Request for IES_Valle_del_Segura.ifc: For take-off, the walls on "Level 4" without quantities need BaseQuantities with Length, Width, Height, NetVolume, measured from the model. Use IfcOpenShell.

First a look at what the model holds.

```python
import ifcopenshell
import ifcopenshell.util.element
import ifcopenshell.util.unit

model = ifcopenshell.open("IES_Valle_del_Segura.ifc")
print(model.schema)
for unit_type in ("LENGTHUNIT", "AREAUNIT", "VOLUMEUNIT"):
    print(unit_type, ifcopenshell.util.unit.calculate_unit_scale(model, unit_type))
storey = next(s for s in model.by_type("IfcBuildingStorey") if s.Name == "Level 4")
walls = [e for e in ifcopenshell.util.element.get_decomposition(storey) if e.is_a("IfcWall")]
for e in sorted(walls, key=lambda e: e.id()):
    print(e.id(), e.is_a(), e.Name, list(ifcopenshell.util.element.get_psets(e, qtos_only=True)), sep=" | ")
```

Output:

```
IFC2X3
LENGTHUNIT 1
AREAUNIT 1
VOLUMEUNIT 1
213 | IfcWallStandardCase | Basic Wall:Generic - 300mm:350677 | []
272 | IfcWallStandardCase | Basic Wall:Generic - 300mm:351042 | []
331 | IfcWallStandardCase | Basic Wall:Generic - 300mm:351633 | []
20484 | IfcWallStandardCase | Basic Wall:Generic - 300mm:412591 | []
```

```python
import ifcopenshell
import ifcopenshell.api.pset
import ifcopenshell.geom
import ifcopenshell.util.element
import ifcopenshell.util.shape
import ifcopenshell.util.unit

model = ifcopenshell.open("IES_Valle_del_Segura.ifc")
unit_scale = ifcopenshell.util.unit.calculate_unit_scale(model)
volume_scale = ifcopenshell.util.unit.calculate_unit_scale(model, "VOLUMEUNIT")
settings = ifcopenshell.geom.settings()

storey = next(s for s in model.by_type("IfcBuildingStorey") if s.Name == "Level 4")
walls = [e for e in ifcopenshell.util.element.get_decomposition(storey) if e.is_a("IfcWall")]

for e in sorted(walls, key=lambda e: e.id()):
    if ifcopenshell.util.element.get_psets(e, qtos_only=True, should_inherit=False):
        continue
    # Geometry comes back in metres, in the element's own axes.
    shape = ifcopenshell.geom.create_shape(settings, e)
    values = {
        "Length": ifcopenshell.util.shape.get_x(shape.geometry) / unit_scale,
        "Width": ifcopenshell.util.shape.get_y(shape.geometry) / unit_scale,
        "Height": ifcopenshell.util.shape.get_z(shape.geometry) / unit_scale,
        "NetVolume": ifcopenshell.util.shape.get_volume(shape.geometry) / volume_scale,
    }
    qto = ifcopenshell.api.pset.add_qto(model, product=e, name="BaseQuantities")
    ifcopenshell.api.pset.edit_qto(model, qto=qto, properties=values)
    print(e.id(), {k: round(v, 3) for k, v in values.items()})

model.write("IES_Valle_del_Segura_v2.ifc")
```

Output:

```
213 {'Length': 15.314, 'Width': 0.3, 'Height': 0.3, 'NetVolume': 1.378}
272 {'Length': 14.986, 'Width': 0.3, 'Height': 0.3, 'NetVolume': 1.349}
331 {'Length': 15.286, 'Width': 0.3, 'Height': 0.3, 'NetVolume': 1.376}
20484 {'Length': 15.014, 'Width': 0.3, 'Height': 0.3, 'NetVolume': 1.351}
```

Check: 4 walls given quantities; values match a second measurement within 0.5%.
